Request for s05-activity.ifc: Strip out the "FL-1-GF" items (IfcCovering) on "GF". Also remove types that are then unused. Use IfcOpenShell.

First a look at what the model holds.

```python
import ifcopenshell
import ifcopenshell.util.element

model = ifcopenshell.open("s05-activity.ifc")
print(model.schema)
storey = next(s for s in model.by_type("IfcBuildingStorey") if s.Name == "GF")
coverings = [e for e in ifcopenshell.util.element.get_decomposition(storey) if e.is_a("IfcCovering")]
seen = {}
for e in coverings:
    element_type = ifcopenshell.util.element.get_type(e)
    name = element_type.Name if element_type not in (None, e) else None
    seen[name] = seen.get(name, 0) + 1
for name, count in sorted(seen.items(), key=str):
    print(count, "x", name)
```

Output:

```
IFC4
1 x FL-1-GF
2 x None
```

```python
import ifcopenshell
import ifcopenshell.api.root
import ifcopenshell.util.element

model = ifcopenshell.open("s05-activity.ifc")

storey = next(s for s in model.by_type("IfcBuildingStorey") if s.Name == "GF")
coverings = [e for e in ifcopenshell.util.element.get_decomposition(storey) if e.is_a("IfcCovering")]
targets = [e for e in coverings if (t := ifcopenshell.util.element.get_type(e)) not in (None, e) and t.Name == "FL-1-GF"]
types = {ifcopenshell.util.element.get_type(e) for e in targets} - {None, *targets}

for e in targets:
    ifcopenshell.api.root.remove_product(model, product=e)
print(len(targets), "removed")

unused = [t for t in types if not ifcopenshell.util.element.get_types(t)]
for t in unused:
    ifcopenshell.api.root.remove_product(model, product=t)
print(len(unused), "unused types removed")

model.write("s05-activity-out.ifc")
```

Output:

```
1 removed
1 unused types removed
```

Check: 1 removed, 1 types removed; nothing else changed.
